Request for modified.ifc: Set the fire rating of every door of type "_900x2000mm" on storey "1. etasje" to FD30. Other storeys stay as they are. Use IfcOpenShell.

First a look at what the model holds.

```python
import ifcopenshell
import ifcopenshell.util.element

model = ifcopenshell.open("modified.ifc")
print(model.schema)
storey = next(s for s in model.by_type("IfcBuildingStorey") if s.Name == "1. etasje")
doors = [e for e in ifcopenshell.util.element.get_decomposition(storey) if e.is_a("IfcDoor")]
seen = {}
for e in doors:
    element_type = ifcopenshell.util.element.get_type(e)
    key = (element_type.Name if element_type != e and element_type else None, ifcopenshell.util.element.get_pset(e, "Pset_DoorCommon", "FireRating"))
    seen[key] = seen.get(key, 0) + 1
for (name, value), count in sorted(seen.items(), key=str):
    print(count, "x", name, "|", value)
```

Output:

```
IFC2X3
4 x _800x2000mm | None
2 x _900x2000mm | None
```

```python
import ifcopenshell
import ifcopenshell.api.pset
import ifcopenshell.util.element

model = ifcopenshell.open("modified.ifc")

storey = next(s for s in model.by_type("IfcBuildingStorey") if s.Name == "1. etasje")
doors = [e for e in ifcopenshell.util.element.get_decomposition(storey) if e.is_a("IfcDoor")]

count = 0
for e in doors:
    element_type = ifcopenshell.util.element.get_type(e)
    if element_type in (None, e) or element_type.Name != "_900x2000mm":
        continue
    # add_pset returns the element's existing set when there is one.
    pset = ifcopenshell.api.pset.add_pset(model, product=e, name="Pset_DoorCommon")
    ifcopenshell.api.pset.edit_pset(model, pset=pset, properties={"FireRating": "FD30"})
    count += 1

print(count, "doors updated")

model.write("modified-out.ifc")
```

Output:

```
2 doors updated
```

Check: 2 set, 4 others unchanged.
